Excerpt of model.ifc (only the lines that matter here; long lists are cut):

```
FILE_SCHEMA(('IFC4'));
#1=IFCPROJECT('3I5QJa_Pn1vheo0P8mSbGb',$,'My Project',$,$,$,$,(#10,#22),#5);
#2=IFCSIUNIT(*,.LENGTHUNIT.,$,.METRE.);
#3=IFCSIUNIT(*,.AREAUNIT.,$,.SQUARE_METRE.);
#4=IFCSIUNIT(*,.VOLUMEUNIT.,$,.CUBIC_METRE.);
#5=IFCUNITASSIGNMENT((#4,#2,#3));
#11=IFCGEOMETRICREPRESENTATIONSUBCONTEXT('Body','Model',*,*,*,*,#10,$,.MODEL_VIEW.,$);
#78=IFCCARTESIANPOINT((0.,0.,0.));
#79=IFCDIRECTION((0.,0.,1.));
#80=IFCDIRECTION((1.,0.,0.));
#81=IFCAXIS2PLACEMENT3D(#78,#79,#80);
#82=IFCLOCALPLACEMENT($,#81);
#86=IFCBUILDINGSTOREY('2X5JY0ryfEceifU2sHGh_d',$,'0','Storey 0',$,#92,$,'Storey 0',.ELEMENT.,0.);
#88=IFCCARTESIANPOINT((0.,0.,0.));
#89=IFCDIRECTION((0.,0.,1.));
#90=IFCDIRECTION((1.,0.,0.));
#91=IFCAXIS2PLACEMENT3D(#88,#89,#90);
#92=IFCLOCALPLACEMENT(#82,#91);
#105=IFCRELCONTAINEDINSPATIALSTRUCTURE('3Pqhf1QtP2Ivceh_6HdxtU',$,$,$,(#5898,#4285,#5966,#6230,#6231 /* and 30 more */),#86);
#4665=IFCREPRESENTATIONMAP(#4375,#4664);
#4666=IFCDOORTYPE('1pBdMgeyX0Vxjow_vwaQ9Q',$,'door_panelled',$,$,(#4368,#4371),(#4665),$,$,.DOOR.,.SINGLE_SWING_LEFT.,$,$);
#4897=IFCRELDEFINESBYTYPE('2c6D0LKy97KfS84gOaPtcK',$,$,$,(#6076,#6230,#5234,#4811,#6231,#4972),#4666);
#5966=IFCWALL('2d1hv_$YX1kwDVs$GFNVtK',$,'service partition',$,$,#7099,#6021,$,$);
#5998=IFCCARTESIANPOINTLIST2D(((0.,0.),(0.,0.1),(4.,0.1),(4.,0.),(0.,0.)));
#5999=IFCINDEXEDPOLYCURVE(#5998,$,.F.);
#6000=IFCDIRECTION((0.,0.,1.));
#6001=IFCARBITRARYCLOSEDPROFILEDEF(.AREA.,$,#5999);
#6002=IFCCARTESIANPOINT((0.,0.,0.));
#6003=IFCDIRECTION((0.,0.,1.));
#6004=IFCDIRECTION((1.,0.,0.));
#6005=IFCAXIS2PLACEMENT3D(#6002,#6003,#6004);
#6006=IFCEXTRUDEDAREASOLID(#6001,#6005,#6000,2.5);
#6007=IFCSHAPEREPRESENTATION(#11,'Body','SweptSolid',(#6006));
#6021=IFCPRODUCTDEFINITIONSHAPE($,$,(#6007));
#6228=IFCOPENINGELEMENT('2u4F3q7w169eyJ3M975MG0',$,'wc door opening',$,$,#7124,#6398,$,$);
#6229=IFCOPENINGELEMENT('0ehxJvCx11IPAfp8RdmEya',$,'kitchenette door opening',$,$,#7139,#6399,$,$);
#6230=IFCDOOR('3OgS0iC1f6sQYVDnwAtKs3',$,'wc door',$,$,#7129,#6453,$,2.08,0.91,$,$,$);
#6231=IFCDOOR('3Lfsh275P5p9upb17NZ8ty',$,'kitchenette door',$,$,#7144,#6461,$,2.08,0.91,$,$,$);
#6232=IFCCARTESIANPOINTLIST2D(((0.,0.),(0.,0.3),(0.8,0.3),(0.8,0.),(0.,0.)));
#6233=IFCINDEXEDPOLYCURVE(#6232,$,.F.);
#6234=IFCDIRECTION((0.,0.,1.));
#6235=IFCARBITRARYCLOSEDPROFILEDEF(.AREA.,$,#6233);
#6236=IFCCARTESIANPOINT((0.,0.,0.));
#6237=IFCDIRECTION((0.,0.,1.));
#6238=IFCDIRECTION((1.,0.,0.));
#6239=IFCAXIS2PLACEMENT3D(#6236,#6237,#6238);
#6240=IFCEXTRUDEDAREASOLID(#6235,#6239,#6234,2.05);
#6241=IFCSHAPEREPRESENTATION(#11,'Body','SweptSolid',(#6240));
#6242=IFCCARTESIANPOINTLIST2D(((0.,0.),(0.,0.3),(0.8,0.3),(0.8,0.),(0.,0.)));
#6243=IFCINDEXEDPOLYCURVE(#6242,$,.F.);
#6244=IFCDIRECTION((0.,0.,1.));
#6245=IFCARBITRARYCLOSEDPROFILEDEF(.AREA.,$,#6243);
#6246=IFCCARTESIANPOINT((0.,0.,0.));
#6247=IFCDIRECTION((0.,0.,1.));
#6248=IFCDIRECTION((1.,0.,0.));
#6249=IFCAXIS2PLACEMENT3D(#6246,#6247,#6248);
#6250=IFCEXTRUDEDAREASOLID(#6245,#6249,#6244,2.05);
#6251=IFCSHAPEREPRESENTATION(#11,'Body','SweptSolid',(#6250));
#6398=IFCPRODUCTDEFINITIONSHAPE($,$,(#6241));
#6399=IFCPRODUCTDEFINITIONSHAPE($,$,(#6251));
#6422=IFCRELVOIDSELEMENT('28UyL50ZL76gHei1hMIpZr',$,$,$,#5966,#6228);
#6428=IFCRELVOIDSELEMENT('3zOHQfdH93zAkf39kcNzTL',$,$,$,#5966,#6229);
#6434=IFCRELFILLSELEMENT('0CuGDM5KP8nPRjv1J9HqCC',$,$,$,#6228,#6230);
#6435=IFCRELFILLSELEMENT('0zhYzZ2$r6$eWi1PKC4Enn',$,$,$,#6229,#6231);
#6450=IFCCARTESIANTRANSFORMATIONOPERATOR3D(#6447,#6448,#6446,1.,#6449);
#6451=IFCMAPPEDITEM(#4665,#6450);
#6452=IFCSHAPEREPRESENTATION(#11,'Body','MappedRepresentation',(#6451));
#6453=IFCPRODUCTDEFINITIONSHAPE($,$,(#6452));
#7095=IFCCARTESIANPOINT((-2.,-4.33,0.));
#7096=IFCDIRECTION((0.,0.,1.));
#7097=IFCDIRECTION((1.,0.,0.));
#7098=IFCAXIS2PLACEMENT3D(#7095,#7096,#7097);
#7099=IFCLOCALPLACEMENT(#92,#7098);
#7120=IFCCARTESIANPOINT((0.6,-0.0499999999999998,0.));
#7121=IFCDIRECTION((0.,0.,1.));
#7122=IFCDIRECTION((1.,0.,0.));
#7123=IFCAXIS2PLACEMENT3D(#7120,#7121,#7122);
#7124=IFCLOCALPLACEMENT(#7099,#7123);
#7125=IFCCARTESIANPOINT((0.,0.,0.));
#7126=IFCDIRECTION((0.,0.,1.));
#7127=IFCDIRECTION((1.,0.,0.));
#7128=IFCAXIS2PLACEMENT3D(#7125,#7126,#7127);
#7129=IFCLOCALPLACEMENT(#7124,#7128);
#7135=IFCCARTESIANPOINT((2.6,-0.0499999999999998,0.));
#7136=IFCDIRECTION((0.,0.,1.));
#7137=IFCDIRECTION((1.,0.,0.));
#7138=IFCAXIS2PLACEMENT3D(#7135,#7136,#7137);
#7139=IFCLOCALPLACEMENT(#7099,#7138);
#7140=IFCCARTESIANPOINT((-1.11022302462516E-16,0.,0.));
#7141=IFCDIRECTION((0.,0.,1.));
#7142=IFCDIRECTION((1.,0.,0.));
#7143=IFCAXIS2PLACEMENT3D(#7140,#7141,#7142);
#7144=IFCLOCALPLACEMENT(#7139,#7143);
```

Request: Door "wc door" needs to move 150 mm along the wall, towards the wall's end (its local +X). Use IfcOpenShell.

```python
import ifcopenshell
import ifcopenshell.api.geometry
import ifcopenshell.util.placement

model = ifcopenshell.open("model.ifc")

door = model.by_id(6230)
opening = door.FillsVoids[0].RelatingOpeningElement
wall = opening.VoidsElements[0].RelatingBuildingElement

wall_matrix = ifcopenshell.util.placement.get_local_placement(wall.ObjectPlacement)
shift = wall_matrix[:3, 0] * 0.15
before = ifcopenshell.util.placement.get_local_placement(door.ObjectPlacement)[:3, 3].copy()

# The door is placed relative to its opening, so it follows when the opening moves.
matrix = ifcopenshell.util.placement.get_local_placement(opening.ObjectPlacement)
matrix[:3, 3] += shift
ifcopenshell.api.geometry.edit_object_placement(
    model, product=opening, matrix=matrix, is_si=False, should_transform_children=True
)

after = ifcopenshell.util.placement.get_local_placement(door.ObjectPlacement)[:3, 3]
print("door moved by", (after - before).round(3) + 0.0)

model.write("model_edited.ifc")
```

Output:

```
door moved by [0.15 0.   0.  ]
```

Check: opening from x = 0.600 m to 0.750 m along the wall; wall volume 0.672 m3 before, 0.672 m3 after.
